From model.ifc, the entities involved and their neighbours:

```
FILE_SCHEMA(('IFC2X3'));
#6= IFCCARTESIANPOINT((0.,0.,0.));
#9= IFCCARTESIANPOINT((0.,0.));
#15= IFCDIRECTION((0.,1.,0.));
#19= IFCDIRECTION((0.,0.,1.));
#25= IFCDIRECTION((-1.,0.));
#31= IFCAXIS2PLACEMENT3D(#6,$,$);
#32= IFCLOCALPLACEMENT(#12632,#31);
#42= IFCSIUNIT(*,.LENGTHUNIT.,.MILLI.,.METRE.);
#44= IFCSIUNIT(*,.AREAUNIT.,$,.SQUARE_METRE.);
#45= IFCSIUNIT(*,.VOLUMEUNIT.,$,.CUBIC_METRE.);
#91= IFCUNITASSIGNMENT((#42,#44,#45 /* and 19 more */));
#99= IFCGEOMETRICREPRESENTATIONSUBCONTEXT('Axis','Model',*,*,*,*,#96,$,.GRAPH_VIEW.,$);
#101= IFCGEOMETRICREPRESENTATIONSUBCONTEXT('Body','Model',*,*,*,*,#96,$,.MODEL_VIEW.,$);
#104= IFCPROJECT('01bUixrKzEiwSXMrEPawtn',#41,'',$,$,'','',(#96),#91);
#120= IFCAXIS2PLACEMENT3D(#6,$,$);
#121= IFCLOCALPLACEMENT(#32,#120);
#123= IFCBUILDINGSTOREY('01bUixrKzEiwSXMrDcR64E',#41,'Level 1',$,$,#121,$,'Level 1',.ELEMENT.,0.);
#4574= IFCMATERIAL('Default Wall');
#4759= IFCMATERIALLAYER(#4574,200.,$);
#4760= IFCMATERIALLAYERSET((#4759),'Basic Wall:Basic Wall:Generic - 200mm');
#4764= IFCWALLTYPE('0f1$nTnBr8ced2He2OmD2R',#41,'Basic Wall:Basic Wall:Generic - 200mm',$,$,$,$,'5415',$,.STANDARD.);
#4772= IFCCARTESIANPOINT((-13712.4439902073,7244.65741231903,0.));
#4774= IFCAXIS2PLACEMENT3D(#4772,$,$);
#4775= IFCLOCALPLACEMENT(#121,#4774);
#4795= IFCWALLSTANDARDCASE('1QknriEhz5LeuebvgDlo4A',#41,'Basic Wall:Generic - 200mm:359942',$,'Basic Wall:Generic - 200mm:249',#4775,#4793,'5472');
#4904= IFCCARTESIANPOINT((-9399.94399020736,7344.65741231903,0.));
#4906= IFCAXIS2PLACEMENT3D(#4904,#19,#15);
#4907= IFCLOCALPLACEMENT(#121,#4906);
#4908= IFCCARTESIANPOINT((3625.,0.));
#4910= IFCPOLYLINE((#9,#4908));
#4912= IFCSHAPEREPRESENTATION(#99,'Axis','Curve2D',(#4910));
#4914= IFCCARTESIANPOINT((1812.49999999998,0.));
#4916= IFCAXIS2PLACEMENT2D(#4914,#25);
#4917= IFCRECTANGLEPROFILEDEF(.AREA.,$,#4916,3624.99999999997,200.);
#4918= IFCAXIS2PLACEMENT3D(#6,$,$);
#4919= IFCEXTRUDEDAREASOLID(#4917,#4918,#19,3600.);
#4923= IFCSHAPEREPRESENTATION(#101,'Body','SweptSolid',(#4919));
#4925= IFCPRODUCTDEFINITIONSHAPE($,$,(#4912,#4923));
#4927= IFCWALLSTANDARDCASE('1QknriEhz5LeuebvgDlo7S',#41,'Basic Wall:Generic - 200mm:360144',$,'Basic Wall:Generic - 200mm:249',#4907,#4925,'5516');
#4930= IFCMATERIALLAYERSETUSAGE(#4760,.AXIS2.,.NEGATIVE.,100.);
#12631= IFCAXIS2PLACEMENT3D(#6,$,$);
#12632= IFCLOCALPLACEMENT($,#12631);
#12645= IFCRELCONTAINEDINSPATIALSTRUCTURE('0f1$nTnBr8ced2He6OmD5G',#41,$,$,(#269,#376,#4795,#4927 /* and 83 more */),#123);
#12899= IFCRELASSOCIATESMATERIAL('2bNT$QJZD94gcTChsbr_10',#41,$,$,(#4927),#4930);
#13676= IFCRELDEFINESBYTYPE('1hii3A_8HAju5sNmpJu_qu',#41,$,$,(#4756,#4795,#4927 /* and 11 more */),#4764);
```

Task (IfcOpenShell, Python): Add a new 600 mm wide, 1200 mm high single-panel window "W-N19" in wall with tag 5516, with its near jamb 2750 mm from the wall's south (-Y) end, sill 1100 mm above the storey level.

```python
import numpy as np
import ifcopenshell
import ifcopenshell.api.feature
import ifcopenshell.api.geometry
import ifcopenshell.api.root
import ifcopenshell.api.spatial
import ifcopenshell.api.type
import ifcopenshell.geom
import ifcopenshell.util.element
import ifcopenshell.util.placement
import ifcopenshell.util.representation
import ifcopenshell.util.shape
import ifcopenshell.util.unit

model = ifcopenshell.open("model.ifc")
unit_scale = ifcopenshell.util.unit.calculate_unit_scale(model)
settings = ifcopenshell.geom.settings()


def volume(element):
    """Net volume in cubic metres, openings subtracted."""
    shape = ifcopenshell.geom.create_shape(settings, element)
    return ifcopenshell.util.shape.get_volume(shape.geometry)


wall = model.by_id(4927)
storey = ifcopenshell.util.element.get_container(wall, ifc_class="IfcBuildingStorey")
context = ifcopenshell.util.representation.get_context(model, "Model", "Body", "MODEL_VIEW")
before = volume(wall)

width, height, from_end, sill = 0.6, 1.2, 2.75, 1.1  # metres

# The wall runs along its own X axis, and the end named is its -X end.
wall_shape = ifcopenshell.geom.create_shape(settings, wall)
x, y, z = ifcopenshell.util.shape.get_vertices(wall_shape.geometry).T
start = x.min() + from_end
face, thickness = float(y.min()), float(y.max() - y.min())
wall_matrix = ifcopenshell.util.placement.get_local_placement(wall.ObjectPlacement)
level = ifcopenshell.util.placement.get_local_placement(storey.ObjectPlacement)[2, 3]


def in_wall(x, y):
    """Placement at x, y metres in the wall's axes, at sill height."""
    matrix = wall_matrix.copy()
    matrix[:, 3] = wall_matrix @ np.array([x / unit_scale, y / unit_scale, 0.0, 1.0])
    matrix[2, 3] = level + sill / unit_scale
    return matrix


# Opening: a box that overshoots both wall faces by 50 mm.
opening = ifcopenshell.api.root.create_entity(model, ifc_class="IfcOpeningElement")
box = ifcopenshell.api.geometry.add_wall_representation(
    model, context=context, length=width, height=height, thickness=thickness + 0.1
)
ifcopenshell.api.geometry.assign_representation(model, product=opening, representation=box)
ifcopenshell.api.geometry.edit_object_placement(model, product=opening, matrix=in_wall(start, face - 0.05), is_si=False)
ifcopenshell.api.feature.add_feature(model, feature=opening, element=wall)

window = ifcopenshell.api.root.create_entity(model, ifc_class="IfcWindow", name="W-N19")
window.OverallWidth, window.OverallHeight = width / unit_scale, height / unit_scale
body = ifcopenshell.api.geometry.add_window_representation(
    model,
    context=context,
    overall_width=window.OverallWidth,
    overall_height=window.OverallHeight,
    partition_type="SINGLE_PANEL",
)
ifcopenshell.api.geometry.assign_representation(model, product=window, representation=body)
ifcopenshell.api.spatial.assign_container(model, products=[window], relating_structure=storey)
fills = ifcopenshell.api.feature.add_filling(model, opening=opening, element=window)
fills.OwnerHistory = window.OwnerHistory  # required in IFC2X3

# IFC2X3 keeps the operation on the window style.
style = ifcopenshell.api.root.create_entity(model, ifc_class="IfcWindowStyle", name="W-N19")
style.OperationType, style.ConstructionType = "SINGLE_PANEL", "NOTDEFINED"
style.ParameterTakesPrecedence = style.Sizeable = False
ifcopenshell.api.type.assign_type(model, related_objects=[window], relating_type=style)

# Centre the window in the wall's thickness.
ifcopenshell.api.geometry.edit_object_placement(model, product=window, matrix=in_wall(start, face), is_si=False)
window_shape = ifcopenshell.geom.create_shape(settings, window)
depth = ifcopenshell.util.shape.get_vertices(window_shape.geometry)[:, 1]
offset = face + thickness / 2 - (depth.min() + depth.max()) / 2
ifcopenshell.api.geometry.edit_object_placement(model, product=window, matrix=in_wall(start, offset), is_si=False)

after = volume(wall)

print(f"wall volume {before:.3f} -> {after:.3f} m3")

model.write("model_updated.ifc")
```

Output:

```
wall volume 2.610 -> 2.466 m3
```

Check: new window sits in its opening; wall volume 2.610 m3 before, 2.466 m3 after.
